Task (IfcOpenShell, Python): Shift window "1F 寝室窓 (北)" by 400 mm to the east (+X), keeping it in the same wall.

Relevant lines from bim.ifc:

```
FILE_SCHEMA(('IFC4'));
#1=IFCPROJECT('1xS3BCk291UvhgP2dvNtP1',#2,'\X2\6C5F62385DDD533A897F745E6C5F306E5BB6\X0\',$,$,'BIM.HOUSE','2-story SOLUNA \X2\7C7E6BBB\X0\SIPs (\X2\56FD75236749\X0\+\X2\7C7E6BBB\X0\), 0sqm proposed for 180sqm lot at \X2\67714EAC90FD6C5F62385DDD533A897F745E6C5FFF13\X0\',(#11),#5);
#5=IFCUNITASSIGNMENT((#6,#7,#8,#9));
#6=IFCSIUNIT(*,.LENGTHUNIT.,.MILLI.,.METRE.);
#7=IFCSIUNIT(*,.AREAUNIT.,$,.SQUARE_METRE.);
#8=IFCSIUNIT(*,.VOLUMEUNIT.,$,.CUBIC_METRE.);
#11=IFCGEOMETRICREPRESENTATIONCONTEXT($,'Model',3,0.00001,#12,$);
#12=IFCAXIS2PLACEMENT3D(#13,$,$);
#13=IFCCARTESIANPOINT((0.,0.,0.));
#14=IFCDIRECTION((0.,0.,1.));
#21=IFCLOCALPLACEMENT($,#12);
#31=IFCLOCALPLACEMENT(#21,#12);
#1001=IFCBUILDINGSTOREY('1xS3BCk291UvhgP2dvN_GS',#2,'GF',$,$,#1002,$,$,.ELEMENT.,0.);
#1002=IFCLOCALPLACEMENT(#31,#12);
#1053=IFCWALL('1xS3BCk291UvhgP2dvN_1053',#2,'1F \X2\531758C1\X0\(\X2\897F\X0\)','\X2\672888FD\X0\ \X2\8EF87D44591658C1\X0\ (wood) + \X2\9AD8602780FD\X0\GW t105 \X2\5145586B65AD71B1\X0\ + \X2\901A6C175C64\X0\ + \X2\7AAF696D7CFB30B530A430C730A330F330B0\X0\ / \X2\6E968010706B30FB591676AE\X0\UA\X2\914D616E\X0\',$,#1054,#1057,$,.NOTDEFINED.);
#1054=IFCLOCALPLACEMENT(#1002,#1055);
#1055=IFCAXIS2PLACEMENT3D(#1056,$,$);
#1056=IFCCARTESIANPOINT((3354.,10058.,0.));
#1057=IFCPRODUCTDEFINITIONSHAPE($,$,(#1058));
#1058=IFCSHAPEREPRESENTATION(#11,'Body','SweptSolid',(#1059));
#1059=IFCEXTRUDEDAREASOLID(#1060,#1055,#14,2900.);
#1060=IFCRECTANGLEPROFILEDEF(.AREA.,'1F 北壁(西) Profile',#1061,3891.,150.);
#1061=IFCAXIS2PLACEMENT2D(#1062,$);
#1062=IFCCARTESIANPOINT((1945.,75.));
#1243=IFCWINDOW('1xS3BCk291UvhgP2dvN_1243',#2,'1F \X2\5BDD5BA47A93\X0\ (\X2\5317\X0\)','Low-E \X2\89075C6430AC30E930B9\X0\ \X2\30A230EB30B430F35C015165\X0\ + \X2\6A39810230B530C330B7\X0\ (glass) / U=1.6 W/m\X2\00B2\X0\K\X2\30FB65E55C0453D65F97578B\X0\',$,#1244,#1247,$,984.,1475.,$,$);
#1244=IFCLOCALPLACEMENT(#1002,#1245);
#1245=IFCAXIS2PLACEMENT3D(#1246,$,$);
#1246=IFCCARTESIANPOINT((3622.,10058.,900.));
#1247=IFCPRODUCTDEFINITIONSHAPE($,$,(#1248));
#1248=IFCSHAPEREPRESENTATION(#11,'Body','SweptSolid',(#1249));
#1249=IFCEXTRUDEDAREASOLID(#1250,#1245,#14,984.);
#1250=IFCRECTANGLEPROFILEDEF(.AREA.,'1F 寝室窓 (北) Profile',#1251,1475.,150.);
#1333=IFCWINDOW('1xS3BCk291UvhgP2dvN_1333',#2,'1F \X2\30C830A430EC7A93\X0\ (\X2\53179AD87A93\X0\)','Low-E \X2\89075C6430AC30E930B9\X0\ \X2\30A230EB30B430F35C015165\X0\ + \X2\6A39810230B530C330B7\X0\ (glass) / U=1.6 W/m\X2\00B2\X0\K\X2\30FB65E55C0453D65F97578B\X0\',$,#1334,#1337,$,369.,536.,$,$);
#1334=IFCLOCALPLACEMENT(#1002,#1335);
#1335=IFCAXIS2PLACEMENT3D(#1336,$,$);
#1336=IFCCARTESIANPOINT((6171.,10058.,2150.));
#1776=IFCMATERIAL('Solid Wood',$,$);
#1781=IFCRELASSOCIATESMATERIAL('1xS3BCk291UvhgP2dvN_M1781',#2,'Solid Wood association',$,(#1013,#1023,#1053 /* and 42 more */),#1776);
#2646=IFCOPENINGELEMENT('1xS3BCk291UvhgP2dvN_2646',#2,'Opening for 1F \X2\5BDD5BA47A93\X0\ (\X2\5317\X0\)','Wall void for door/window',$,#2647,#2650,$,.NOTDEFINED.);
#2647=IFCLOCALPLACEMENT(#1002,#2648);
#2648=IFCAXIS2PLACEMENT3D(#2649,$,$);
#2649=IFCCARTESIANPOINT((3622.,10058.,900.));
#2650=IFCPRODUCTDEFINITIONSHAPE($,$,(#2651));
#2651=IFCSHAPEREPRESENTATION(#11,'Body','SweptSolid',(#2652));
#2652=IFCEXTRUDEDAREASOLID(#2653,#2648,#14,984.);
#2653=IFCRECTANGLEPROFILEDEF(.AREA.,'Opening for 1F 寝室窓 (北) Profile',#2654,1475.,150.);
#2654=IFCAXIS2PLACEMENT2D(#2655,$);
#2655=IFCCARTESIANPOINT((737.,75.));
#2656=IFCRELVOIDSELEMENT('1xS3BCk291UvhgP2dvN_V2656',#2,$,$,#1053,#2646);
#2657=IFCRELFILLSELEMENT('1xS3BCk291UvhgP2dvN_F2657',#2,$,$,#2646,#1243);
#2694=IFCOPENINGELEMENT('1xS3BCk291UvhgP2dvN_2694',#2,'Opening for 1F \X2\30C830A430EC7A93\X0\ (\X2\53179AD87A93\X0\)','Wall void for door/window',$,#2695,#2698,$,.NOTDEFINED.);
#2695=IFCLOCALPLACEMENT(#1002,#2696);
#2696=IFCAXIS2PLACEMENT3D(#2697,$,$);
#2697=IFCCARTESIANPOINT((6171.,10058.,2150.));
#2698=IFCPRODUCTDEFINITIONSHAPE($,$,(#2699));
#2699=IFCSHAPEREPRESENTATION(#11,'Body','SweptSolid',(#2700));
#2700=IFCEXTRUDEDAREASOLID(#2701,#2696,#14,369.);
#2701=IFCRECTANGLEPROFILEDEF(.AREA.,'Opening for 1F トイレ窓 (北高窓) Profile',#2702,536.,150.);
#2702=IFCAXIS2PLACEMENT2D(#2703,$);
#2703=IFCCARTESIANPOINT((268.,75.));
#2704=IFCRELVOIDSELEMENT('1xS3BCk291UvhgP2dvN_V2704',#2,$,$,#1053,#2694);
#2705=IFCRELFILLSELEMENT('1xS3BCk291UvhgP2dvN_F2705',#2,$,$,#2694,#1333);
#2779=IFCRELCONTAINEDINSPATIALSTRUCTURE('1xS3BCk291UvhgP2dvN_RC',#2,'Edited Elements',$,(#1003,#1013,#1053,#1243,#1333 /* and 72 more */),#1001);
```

```python
import ifcopenshell
import ifcopenshell.api.geometry
import ifcopenshell.util.placement

model = ifcopenshell.open("bim.ifc")

window = model.by_guid("1xS3BCk291UvhgP2dvN_1243")
opening = window.FillsVoids[0].RelatingOpeningElement
wall = opening.VoidsElements[0].RelatingBuildingElement

wall_matrix = ifcopenshell.util.placement.get_local_placement(wall.ObjectPlacement)
shift = wall_matrix[:3, 0] * 400.0
before = ifcopenshell.util.placement.get_local_placement(window.ObjectPlacement)[:3, 3].copy()

# The window is not placed relative to its opening, so move both.
for product in (opening, window):
    matrix = ifcopenshell.util.placement.get_local_placement(product.ObjectPlacement)
    matrix[:3, 3] += shift
    ifcopenshell.api.geometry.edit_object_placement(model, product=product, matrix=matrix, is_si=False)

after = ifcopenshell.util.placement.get_local_placement(window.ObjectPlacement)[:3, 3]
print("window moved by", (after - before).round(3) + 0.0)

model.write("bim_rev.ifc")
```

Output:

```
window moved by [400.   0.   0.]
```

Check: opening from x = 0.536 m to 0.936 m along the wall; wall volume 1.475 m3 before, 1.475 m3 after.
